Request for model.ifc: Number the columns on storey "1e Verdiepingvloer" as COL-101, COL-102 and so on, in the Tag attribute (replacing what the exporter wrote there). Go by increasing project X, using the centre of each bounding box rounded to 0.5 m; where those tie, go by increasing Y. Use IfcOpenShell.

First a look at what the model holds.

```python
import ifcopenshell
import ifcopenshell.util.element
import ifcopenshell.util.placement

model = ifcopenshell.open("model.ifc")
print(model.schema)
storey = next(s for s in model.by_type("IfcBuildingStorey") if s.Name == "1e Verdiepingvloer")
columns = [e for e in ifcopenshell.util.element.get_decomposition(storey) if e.is_a("IfcColumn")]
for e in sorted(columns, key=lambda e: e.id()):
    origin = ifcopenshell.util.placement.get_local_placement(e.ObjectPlacement)[:3, 3]
    print(e.id(), e.Tag, e.Name, origin.round(2) + 0.0, sep=" | ")
```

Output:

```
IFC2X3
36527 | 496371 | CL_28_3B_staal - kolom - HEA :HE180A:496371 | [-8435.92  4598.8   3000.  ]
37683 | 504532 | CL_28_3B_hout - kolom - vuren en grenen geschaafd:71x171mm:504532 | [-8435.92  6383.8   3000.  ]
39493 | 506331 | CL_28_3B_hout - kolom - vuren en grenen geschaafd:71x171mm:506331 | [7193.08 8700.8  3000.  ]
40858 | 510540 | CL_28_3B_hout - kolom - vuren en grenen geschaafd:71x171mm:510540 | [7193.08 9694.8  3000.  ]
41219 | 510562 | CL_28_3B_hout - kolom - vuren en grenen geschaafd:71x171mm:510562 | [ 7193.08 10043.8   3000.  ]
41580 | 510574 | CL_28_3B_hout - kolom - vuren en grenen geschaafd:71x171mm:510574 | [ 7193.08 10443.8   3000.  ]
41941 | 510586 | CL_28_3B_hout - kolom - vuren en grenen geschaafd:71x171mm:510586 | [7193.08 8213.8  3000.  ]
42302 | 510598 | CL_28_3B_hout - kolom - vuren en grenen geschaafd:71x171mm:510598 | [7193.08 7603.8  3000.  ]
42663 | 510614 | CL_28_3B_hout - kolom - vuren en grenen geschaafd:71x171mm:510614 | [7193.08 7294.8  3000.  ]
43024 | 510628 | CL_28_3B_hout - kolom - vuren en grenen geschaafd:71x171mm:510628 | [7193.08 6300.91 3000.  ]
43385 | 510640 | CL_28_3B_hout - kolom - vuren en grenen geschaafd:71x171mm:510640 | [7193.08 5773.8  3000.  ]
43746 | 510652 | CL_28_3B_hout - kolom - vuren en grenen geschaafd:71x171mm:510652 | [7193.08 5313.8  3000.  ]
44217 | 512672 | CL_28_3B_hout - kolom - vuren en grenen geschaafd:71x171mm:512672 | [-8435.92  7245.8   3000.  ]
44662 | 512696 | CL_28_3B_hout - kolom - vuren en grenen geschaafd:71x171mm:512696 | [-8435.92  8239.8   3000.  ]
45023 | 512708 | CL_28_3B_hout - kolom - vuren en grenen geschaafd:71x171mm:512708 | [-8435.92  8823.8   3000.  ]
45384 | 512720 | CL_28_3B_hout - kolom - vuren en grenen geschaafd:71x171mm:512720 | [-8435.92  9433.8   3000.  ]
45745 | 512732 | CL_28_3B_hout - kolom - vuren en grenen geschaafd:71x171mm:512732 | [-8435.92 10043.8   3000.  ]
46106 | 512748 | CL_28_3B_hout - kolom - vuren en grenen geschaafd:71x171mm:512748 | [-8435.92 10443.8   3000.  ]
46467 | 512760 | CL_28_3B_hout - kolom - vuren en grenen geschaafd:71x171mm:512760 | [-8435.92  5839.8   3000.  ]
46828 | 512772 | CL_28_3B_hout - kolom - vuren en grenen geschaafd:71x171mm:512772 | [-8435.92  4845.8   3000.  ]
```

```python
import ifcopenshell
import ifcopenshell.geom
import ifcopenshell.util.element
import ifcopenshell.util.shape

model = ifcopenshell.open("model.ifc")
settings = ifcopenshell.geom.settings()
settings.set("use-world-coords", True)


def centre(element):
    shape = ifcopenshell.geom.create_shape(settings, element)
    return ifcopenshell.util.shape.get_bbox_centroid(shape.geometry)


storey = next(s for s in model.by_type("IfcBuildingStorey") if s.Name == "1e Verdiepingvloer")
columns = [e for e in ifcopenshell.util.element.get_decomposition(storey) if e.is_a("IfcColumn")]

# Insertion points can sit at a corner or the storey origin, so sort by the geometry (in metres).
centres = {e: centre(e) for e in columns}
columns.sort(key=lambda e: (round(centres[e][0] / 0.5), centres[e][1]))

for i, e in enumerate(columns, start=1):
    number = f"COL-1{i:02d}"
    e.Tag = number
    print(e.id(), number)

model.write("model-out.ifc")
```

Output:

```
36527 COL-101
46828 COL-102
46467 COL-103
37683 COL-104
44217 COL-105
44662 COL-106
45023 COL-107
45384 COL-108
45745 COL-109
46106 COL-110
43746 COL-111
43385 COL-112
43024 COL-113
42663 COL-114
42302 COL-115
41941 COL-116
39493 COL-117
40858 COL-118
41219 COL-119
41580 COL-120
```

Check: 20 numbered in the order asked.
